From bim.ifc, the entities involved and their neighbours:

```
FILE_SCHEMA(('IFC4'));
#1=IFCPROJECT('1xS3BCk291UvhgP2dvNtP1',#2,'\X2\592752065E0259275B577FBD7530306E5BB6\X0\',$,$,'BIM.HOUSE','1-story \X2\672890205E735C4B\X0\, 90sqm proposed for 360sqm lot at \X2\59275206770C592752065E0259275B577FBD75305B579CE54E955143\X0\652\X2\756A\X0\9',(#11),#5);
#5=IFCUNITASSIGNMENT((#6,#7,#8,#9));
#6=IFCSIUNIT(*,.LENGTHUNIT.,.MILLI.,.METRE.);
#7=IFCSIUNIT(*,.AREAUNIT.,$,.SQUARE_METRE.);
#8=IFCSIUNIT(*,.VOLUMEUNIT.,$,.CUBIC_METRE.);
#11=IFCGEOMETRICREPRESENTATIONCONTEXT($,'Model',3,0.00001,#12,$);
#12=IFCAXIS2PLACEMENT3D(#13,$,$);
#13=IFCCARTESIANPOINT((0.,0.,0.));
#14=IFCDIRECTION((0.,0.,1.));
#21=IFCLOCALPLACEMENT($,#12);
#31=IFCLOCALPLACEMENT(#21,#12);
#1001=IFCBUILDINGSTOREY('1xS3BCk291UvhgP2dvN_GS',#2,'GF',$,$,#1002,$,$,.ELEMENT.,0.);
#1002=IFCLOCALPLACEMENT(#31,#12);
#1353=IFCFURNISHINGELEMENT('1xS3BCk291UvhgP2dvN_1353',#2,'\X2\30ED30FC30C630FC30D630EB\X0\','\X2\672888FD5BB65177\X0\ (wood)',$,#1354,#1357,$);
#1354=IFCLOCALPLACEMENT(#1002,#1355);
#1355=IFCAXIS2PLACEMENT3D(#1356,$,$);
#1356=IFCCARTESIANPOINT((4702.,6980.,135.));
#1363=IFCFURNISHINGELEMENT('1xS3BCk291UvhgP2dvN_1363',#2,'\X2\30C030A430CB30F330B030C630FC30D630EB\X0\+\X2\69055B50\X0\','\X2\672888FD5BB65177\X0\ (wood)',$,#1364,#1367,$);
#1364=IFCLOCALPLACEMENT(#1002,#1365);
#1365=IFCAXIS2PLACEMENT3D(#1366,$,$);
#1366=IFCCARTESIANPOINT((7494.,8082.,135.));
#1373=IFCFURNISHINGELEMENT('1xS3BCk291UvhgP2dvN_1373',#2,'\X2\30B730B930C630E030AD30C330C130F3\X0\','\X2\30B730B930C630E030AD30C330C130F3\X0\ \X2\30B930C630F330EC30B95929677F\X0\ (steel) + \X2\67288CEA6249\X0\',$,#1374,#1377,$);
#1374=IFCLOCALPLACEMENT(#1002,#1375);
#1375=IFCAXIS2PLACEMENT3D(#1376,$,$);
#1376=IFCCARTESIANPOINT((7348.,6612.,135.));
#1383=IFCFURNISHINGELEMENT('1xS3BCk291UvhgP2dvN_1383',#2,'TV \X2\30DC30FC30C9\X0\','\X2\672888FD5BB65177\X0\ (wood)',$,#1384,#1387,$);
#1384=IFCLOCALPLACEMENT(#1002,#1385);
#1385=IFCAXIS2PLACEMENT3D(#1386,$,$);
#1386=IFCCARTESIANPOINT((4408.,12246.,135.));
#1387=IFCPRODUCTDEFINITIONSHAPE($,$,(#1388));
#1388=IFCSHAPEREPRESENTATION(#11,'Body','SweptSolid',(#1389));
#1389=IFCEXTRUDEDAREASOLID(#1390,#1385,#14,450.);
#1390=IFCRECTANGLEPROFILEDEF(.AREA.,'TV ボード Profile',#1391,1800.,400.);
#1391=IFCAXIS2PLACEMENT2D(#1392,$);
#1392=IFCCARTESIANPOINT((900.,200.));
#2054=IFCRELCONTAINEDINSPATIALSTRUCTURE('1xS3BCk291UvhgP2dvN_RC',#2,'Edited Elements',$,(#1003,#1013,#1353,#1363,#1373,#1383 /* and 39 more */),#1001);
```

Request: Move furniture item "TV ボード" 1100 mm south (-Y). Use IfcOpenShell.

```python
import ifcopenshell
import ifcopenshell.api.geometry
import ifcopenshell.util.placement
import ifcopenshell.util.unit

model = ifcopenshell.open("bim.ifc")
unit_scale = ifcopenshell.util.unit.calculate_unit_scale(model)

item = model.by_guid("1xS3BCk291UvhgP2dvN_1383")
matrix = ifcopenshell.util.placement.get_local_placement(item.ObjectPlacement)
matrix[1, 3] -= 1.1 / unit_scale
ifcopenshell.api.geometry.edit_object_placement(model, product=item, matrix=matrix, is_si=False)

print(ifcopenshell.util.placement.get_local_placement(item.ObjectPlacement).round(3) + 0.0)

model.write("bim_edited.ifc")
```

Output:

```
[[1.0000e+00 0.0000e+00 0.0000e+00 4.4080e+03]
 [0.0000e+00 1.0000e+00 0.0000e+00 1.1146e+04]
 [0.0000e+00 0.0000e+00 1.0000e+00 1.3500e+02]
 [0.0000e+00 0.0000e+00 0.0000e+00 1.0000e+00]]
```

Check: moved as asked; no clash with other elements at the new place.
